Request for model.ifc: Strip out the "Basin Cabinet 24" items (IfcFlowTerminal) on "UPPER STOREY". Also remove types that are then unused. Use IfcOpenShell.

First a look at what the model holds.

```python
import ifcopenshell
import ifcopenshell.util.element

model = ifcopenshell.open("model.ifc")
print(model.schema)
storey = next(s for s in model.by_type("IfcBuildingStorey") if s.Name == "UPPER STOREY")
terminals = [e for e in ifcopenshell.util.element.get_decomposition(storey) if e.is_a("IfcFlowTerminal")]
seen = {}
for e in terminals:
    element_type = ifcopenshell.util.element.get_type(e)
    name = element_type.Name if element_type not in (None, e) else None
    seen[name] = seen.get(name, 0) + 1
for name, count in sorted(seen.items(), key=str):
    print(count, "x", name)
```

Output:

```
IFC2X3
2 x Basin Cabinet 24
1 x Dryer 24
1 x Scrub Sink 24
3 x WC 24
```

```python
import ifcopenshell
import ifcopenshell.api.root
import ifcopenshell.util.element

model = ifcopenshell.open("model.ifc")

storey = next(s for s in model.by_type("IfcBuildingStorey") if s.Name == "UPPER STOREY")
terminals = [e for e in ifcopenshell.util.element.get_decomposition(storey) if e.is_a("IfcFlowTerminal")]
targets = [e for e in terminals if (t := ifcopenshell.util.element.get_type(e)) not in (None, e) and t.Name == "Basin Cabinet 24"]
types = {ifcopenshell.util.element.get_type(e) for e in targets} - {None, *targets}

for e in targets:
    ifcopenshell.api.root.remove_product(model, product=e)
print(len(targets), "removed")

unused = [t for t in types if not ifcopenshell.util.element.get_types(t)]
for t in unused:
    ifcopenshell.api.root.remove_product(model, product=t)
print(len(unused), "unused types removed")

model.write("model_edited.ifc")
```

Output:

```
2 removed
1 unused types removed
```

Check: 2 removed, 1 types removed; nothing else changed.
